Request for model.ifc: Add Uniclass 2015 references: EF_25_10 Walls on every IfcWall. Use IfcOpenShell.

First a look at what the model holds.

```python
import ifcopenshell

model = ifcopenshell.open("model.ifc")
print(model.schema)
print("classifications:", [c.Name for c in model.by_type("IfcClassification")])
for ifc_class in ("IfcDoor", "IfcRoof", "IfcStair", "IfcWall", "IfcWindow"):
    print(ifc_class, len(model.by_type(ifc_class)))
```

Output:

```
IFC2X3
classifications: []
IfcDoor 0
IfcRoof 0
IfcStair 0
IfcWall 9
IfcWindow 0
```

```python
import ifcopenshell
import ifcopenshell.api.classification

model = ifcopenshell.open("model.ifc")

# IFC2X3 requires Source and Edition and has no link from the project to the system.
system = model.create_entity("IfcClassification", Source="NBS", Edition="2015", Name="Uniclass 2015")

codes = {
    "IfcWall": ("EF_25_10", "Walls"),
}
for ifc_class, (code, name) in codes.items():
    products = model.by_type(ifc_class)
    ifcopenshell.api.classification.add_reference(
        model, products=products, classification=system, identification=code, name=name
    )
    print(code, len(products))

model.write("model_v2.ifc")
```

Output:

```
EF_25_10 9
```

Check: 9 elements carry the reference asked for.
